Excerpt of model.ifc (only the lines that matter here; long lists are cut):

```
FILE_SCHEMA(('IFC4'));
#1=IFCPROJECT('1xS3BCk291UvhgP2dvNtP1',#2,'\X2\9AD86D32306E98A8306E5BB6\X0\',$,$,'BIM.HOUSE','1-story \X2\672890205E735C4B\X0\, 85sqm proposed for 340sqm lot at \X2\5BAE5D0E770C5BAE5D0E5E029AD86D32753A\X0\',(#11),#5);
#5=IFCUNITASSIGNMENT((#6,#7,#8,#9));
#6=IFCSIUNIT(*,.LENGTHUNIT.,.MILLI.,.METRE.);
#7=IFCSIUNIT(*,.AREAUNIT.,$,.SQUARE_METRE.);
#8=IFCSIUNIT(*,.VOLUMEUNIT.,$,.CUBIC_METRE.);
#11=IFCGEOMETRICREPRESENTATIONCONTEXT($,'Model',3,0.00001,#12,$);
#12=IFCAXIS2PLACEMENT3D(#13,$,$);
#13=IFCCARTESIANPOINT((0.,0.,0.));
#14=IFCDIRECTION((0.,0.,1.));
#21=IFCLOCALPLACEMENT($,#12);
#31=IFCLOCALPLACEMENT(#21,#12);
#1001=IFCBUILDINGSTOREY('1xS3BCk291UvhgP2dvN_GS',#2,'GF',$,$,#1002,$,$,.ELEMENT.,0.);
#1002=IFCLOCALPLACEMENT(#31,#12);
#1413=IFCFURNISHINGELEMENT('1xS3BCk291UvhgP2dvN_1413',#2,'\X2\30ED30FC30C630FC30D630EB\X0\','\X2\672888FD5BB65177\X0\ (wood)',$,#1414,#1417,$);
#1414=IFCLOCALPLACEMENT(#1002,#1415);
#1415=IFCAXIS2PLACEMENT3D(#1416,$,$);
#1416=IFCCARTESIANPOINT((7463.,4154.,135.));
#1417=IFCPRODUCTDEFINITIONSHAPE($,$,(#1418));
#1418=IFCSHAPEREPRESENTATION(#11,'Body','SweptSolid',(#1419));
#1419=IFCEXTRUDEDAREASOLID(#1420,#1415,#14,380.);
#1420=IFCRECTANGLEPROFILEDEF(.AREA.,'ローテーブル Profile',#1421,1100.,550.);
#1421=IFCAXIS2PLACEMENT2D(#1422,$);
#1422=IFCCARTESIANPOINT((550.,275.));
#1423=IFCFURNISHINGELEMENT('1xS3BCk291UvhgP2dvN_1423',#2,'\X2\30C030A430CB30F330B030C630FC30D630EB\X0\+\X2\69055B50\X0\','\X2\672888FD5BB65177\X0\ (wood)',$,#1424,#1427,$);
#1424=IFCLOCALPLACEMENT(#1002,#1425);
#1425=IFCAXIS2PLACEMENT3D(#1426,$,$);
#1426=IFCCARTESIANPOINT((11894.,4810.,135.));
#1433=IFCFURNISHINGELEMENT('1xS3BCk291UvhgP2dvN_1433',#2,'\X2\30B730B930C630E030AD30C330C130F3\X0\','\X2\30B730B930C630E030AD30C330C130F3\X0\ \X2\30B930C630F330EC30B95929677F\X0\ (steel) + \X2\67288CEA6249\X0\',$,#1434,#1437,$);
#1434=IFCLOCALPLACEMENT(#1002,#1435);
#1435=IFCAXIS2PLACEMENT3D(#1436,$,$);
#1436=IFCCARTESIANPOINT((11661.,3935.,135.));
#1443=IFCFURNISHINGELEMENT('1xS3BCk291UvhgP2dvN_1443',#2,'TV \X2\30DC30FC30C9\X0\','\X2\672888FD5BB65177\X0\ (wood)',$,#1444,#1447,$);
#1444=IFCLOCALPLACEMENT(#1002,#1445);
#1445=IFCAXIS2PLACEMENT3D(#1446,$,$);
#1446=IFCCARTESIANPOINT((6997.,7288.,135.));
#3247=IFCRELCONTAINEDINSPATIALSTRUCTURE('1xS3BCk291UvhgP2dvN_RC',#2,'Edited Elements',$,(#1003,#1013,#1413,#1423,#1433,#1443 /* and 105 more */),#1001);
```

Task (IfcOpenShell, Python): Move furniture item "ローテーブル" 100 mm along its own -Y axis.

```python
import ifcopenshell
import ifcopenshell.api.geometry
import ifcopenshell.util.placement
import ifcopenshell.util.unit

model = ifcopenshell.open("model.ifc")
unit_scale = ifcopenshell.util.unit.calculate_unit_scale(model)

item = model.by_id(1413)
matrix = ifcopenshell.util.placement.get_local_placement(item.ObjectPlacement)
matrix[:3, 3] -= matrix[:3, 1] * 0.1 / unit_scale
ifcopenshell.api.geometry.edit_object_placement(model, product=item, matrix=matrix, is_si=False)

print(ifcopenshell.util.placement.get_local_placement(item.ObjectPlacement).round(3) + 0.0)

model.write("model_edited.ifc")
```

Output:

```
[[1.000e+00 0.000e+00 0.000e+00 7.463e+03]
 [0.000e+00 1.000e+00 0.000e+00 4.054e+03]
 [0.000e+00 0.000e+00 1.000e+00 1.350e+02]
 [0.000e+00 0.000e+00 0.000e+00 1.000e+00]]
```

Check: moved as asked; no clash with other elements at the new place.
